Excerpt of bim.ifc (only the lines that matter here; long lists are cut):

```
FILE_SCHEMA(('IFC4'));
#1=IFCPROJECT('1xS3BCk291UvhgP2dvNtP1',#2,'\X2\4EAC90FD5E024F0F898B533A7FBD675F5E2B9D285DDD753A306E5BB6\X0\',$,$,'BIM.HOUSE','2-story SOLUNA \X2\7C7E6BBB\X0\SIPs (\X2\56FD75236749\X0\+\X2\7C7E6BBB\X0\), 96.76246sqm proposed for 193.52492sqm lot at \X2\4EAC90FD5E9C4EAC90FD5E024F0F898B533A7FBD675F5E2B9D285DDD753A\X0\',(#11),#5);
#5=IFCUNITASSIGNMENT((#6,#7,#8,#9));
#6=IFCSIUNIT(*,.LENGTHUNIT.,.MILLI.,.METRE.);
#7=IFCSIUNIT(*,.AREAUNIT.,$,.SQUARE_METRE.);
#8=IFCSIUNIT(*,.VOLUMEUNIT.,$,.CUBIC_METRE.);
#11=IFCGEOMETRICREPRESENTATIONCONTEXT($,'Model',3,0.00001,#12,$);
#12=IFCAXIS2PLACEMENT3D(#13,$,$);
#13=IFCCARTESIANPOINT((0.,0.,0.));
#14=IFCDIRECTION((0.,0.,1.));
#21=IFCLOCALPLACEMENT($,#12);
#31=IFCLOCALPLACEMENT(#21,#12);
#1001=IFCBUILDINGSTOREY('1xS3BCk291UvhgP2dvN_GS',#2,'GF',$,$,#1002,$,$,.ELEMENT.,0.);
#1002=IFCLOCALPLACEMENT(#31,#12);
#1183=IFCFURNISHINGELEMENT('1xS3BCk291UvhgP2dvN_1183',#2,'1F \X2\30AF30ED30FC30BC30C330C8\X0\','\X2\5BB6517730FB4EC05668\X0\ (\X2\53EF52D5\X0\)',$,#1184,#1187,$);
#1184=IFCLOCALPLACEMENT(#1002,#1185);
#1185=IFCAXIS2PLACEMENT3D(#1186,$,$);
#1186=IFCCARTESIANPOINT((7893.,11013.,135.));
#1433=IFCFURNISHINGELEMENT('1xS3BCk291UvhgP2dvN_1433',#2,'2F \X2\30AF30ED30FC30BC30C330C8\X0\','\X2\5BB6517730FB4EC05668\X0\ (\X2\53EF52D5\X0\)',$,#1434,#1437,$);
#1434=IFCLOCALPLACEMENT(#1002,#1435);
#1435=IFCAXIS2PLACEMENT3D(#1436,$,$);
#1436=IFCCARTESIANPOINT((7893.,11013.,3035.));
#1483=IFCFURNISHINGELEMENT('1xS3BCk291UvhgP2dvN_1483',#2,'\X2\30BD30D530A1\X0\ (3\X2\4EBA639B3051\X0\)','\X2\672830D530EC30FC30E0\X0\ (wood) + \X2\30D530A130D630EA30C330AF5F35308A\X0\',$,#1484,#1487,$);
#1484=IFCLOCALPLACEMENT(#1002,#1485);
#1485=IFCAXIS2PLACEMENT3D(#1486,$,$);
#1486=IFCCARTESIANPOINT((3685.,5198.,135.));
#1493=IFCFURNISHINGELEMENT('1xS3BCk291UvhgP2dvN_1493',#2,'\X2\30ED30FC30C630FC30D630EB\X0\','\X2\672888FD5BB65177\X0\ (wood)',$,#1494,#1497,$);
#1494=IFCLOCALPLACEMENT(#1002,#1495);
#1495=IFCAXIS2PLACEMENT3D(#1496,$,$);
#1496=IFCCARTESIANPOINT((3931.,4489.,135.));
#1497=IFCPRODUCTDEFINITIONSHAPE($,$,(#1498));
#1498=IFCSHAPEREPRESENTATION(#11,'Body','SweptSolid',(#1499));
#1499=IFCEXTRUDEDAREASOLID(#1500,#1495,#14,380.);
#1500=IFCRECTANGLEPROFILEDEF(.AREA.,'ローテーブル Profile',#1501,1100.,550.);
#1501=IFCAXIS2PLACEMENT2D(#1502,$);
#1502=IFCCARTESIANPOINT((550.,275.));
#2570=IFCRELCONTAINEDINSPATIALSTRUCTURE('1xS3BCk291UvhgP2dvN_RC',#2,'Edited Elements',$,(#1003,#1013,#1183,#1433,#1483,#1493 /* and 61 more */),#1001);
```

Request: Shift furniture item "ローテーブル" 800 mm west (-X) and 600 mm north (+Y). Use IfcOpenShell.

```python
import ifcopenshell
import ifcopenshell.api.geometry
import ifcopenshell.util.placement
import ifcopenshell.util.unit

model = ifcopenshell.open("bim.ifc")
unit_scale = ifcopenshell.util.unit.calculate_unit_scale(model)

item = model.by_guid("1xS3BCk291UvhgP2dvN_1493")
matrix = ifcopenshell.util.placement.get_local_placement(item.ObjectPlacement)
matrix[0, 3] -= 0.8 / unit_scale
matrix[1, 3] += 0.6 / unit_scale
ifcopenshell.api.geometry.edit_object_placement(model, product=item, matrix=matrix, is_si=False)

print(ifcopenshell.util.placement.get_local_placement(item.ObjectPlacement).round(3) + 0.0)

model.write("bim_edited.ifc")
```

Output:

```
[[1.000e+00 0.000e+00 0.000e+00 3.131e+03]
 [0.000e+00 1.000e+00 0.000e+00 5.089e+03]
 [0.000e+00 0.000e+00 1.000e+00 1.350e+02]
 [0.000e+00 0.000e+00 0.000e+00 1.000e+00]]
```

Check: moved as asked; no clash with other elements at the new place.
